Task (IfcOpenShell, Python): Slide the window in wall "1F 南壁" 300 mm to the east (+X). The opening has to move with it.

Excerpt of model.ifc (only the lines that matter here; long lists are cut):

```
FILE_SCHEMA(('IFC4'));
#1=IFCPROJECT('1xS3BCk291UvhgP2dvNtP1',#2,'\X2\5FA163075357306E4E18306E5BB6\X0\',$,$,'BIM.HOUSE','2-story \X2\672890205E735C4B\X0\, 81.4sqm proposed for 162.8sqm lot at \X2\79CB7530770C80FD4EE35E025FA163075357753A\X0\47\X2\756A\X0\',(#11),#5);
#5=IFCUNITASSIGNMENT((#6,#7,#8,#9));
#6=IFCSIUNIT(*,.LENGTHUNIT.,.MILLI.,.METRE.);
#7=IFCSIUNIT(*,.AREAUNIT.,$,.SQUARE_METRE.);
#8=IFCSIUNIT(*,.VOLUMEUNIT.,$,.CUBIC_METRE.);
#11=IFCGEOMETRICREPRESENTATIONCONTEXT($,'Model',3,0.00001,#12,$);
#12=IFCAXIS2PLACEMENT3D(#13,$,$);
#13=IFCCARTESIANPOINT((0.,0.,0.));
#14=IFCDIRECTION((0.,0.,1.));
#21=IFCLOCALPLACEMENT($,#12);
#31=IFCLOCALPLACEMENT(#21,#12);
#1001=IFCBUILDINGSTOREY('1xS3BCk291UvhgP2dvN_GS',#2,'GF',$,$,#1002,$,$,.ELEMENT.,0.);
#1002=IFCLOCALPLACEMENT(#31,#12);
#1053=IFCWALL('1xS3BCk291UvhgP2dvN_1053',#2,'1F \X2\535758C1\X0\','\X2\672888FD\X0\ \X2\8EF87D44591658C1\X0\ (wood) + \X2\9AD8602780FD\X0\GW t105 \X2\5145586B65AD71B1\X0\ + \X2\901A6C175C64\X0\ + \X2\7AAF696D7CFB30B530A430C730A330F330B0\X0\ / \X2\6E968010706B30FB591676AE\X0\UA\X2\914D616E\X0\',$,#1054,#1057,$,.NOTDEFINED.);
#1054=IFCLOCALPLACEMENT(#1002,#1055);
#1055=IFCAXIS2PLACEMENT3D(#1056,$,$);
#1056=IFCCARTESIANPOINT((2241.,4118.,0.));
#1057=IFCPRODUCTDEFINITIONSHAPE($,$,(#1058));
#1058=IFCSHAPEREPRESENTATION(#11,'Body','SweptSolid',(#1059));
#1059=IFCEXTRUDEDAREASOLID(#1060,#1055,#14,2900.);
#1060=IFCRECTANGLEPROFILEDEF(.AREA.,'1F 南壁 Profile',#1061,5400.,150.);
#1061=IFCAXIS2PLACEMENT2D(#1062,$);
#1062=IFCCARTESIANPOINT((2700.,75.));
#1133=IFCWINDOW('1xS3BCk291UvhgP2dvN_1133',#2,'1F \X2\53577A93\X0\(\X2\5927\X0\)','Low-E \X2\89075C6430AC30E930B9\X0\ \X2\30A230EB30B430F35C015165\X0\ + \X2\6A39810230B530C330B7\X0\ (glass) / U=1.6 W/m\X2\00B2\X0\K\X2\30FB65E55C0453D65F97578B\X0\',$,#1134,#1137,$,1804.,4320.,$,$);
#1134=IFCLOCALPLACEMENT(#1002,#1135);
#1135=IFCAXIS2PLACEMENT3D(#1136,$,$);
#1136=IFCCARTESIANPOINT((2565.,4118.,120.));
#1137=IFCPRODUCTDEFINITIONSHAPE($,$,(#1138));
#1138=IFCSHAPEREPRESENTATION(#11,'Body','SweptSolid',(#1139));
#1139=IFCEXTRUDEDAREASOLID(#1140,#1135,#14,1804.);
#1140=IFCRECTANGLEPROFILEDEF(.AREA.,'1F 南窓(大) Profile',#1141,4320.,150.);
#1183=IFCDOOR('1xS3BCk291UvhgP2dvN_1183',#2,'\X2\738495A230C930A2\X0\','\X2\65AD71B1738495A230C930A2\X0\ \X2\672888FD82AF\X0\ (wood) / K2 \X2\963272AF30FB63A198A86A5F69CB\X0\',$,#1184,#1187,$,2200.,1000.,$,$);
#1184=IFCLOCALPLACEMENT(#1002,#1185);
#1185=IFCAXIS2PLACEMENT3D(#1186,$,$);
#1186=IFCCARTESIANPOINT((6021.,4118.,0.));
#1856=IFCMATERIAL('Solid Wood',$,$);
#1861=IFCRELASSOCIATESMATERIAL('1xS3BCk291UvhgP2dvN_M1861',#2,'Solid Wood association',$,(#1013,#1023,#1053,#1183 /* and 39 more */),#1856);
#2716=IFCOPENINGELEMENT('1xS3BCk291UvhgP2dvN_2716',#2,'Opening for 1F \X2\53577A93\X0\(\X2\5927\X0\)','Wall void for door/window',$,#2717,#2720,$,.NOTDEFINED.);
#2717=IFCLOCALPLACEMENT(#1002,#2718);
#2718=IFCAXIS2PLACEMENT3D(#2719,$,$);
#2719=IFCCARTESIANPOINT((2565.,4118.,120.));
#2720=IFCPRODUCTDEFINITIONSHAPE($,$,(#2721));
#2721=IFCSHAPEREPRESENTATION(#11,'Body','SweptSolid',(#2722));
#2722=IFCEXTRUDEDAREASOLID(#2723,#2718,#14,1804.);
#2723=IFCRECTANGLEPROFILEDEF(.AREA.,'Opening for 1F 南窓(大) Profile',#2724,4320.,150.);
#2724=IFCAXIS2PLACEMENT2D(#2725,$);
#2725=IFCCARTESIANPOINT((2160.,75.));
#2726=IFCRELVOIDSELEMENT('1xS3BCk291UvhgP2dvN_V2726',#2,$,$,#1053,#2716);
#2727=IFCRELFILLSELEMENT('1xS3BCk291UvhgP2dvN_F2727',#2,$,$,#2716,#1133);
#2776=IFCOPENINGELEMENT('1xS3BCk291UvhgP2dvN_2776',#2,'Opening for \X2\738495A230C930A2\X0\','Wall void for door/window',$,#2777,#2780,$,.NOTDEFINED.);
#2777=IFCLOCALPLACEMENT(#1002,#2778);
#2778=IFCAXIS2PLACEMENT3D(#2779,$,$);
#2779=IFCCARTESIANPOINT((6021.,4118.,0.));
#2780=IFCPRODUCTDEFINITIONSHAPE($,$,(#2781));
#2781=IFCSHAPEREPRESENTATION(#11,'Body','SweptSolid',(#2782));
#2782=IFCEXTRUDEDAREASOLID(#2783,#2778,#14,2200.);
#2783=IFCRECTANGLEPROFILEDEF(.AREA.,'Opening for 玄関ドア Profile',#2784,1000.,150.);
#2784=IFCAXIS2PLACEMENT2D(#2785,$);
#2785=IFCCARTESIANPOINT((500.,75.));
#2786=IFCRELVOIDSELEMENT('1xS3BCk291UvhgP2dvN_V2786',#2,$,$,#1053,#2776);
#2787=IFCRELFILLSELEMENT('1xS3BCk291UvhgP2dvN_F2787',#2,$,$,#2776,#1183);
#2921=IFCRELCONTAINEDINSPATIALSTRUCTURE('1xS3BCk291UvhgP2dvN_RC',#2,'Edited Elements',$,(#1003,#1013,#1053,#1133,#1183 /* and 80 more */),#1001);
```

```python
import ifcopenshell
import ifcopenshell.api.geometry
import ifcopenshell.util.placement

model = ifcopenshell.open("model.ifc")

window = model.by_id(1133)
opening = window.FillsVoids[0].RelatingOpeningElement
wall = opening.VoidsElements[0].RelatingBuildingElement

wall_matrix = ifcopenshell.util.placement.get_local_placement(wall.ObjectPlacement)
shift = wall_matrix[:3, 0] * 300.0
before = ifcopenshell.util.placement.get_local_placement(window.ObjectPlacement)[:3, 3].copy()

# The window is not placed relative to its opening, so move both.
for product in (opening, window):
    matrix = ifcopenshell.util.placement.get_local_placement(product.ObjectPlacement)
    matrix[:3, 3] += shift
    ifcopenshell.api.geometry.edit_object_placement(model, product=product, matrix=matrix, is_si=False)

after = ifcopenshell.util.placement.get_local_placement(window.ObjectPlacement)[:3, 3]
print("window moved by", (after - before).round(3) + 0.0)

model.write("model_updated.ifc")
```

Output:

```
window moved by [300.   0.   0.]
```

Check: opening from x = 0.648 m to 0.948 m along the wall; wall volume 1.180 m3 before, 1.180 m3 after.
